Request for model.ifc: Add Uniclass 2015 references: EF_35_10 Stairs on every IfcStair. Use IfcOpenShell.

First a look at what the model holds.

```python
import ifcopenshell

model = ifcopenshell.open("model.ifc")
print(model.schema)
print("classifications:", [c.Name for c in model.by_type("IfcClassification")])
for ifc_class in ("IfcDoor", "IfcRoof", "IfcStair", "IfcWall", "IfcWindow"):
    print(ifc_class, len(model.by_type(ifc_class)))
```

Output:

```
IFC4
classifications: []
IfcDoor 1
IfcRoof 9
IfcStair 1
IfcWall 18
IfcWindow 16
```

```python
import ifcopenshell
import ifcopenshell.api.classification

model = ifcopenshell.open("model.ifc")

system = ifcopenshell.api.classification.add_classification(model, classification="Uniclass 2015")

codes = {
    "IfcStair": ("EF_35_10", "Stairs"),
}
for ifc_class, (code, name) in codes.items():
    products = model.by_type(ifc_class)
    ifcopenshell.api.classification.add_reference(
        model, products=products, classification=system, identification=code, name=name
    )
    print(code, len(products))

model.write("model-out.ifc")
```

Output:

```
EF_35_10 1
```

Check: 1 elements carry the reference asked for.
